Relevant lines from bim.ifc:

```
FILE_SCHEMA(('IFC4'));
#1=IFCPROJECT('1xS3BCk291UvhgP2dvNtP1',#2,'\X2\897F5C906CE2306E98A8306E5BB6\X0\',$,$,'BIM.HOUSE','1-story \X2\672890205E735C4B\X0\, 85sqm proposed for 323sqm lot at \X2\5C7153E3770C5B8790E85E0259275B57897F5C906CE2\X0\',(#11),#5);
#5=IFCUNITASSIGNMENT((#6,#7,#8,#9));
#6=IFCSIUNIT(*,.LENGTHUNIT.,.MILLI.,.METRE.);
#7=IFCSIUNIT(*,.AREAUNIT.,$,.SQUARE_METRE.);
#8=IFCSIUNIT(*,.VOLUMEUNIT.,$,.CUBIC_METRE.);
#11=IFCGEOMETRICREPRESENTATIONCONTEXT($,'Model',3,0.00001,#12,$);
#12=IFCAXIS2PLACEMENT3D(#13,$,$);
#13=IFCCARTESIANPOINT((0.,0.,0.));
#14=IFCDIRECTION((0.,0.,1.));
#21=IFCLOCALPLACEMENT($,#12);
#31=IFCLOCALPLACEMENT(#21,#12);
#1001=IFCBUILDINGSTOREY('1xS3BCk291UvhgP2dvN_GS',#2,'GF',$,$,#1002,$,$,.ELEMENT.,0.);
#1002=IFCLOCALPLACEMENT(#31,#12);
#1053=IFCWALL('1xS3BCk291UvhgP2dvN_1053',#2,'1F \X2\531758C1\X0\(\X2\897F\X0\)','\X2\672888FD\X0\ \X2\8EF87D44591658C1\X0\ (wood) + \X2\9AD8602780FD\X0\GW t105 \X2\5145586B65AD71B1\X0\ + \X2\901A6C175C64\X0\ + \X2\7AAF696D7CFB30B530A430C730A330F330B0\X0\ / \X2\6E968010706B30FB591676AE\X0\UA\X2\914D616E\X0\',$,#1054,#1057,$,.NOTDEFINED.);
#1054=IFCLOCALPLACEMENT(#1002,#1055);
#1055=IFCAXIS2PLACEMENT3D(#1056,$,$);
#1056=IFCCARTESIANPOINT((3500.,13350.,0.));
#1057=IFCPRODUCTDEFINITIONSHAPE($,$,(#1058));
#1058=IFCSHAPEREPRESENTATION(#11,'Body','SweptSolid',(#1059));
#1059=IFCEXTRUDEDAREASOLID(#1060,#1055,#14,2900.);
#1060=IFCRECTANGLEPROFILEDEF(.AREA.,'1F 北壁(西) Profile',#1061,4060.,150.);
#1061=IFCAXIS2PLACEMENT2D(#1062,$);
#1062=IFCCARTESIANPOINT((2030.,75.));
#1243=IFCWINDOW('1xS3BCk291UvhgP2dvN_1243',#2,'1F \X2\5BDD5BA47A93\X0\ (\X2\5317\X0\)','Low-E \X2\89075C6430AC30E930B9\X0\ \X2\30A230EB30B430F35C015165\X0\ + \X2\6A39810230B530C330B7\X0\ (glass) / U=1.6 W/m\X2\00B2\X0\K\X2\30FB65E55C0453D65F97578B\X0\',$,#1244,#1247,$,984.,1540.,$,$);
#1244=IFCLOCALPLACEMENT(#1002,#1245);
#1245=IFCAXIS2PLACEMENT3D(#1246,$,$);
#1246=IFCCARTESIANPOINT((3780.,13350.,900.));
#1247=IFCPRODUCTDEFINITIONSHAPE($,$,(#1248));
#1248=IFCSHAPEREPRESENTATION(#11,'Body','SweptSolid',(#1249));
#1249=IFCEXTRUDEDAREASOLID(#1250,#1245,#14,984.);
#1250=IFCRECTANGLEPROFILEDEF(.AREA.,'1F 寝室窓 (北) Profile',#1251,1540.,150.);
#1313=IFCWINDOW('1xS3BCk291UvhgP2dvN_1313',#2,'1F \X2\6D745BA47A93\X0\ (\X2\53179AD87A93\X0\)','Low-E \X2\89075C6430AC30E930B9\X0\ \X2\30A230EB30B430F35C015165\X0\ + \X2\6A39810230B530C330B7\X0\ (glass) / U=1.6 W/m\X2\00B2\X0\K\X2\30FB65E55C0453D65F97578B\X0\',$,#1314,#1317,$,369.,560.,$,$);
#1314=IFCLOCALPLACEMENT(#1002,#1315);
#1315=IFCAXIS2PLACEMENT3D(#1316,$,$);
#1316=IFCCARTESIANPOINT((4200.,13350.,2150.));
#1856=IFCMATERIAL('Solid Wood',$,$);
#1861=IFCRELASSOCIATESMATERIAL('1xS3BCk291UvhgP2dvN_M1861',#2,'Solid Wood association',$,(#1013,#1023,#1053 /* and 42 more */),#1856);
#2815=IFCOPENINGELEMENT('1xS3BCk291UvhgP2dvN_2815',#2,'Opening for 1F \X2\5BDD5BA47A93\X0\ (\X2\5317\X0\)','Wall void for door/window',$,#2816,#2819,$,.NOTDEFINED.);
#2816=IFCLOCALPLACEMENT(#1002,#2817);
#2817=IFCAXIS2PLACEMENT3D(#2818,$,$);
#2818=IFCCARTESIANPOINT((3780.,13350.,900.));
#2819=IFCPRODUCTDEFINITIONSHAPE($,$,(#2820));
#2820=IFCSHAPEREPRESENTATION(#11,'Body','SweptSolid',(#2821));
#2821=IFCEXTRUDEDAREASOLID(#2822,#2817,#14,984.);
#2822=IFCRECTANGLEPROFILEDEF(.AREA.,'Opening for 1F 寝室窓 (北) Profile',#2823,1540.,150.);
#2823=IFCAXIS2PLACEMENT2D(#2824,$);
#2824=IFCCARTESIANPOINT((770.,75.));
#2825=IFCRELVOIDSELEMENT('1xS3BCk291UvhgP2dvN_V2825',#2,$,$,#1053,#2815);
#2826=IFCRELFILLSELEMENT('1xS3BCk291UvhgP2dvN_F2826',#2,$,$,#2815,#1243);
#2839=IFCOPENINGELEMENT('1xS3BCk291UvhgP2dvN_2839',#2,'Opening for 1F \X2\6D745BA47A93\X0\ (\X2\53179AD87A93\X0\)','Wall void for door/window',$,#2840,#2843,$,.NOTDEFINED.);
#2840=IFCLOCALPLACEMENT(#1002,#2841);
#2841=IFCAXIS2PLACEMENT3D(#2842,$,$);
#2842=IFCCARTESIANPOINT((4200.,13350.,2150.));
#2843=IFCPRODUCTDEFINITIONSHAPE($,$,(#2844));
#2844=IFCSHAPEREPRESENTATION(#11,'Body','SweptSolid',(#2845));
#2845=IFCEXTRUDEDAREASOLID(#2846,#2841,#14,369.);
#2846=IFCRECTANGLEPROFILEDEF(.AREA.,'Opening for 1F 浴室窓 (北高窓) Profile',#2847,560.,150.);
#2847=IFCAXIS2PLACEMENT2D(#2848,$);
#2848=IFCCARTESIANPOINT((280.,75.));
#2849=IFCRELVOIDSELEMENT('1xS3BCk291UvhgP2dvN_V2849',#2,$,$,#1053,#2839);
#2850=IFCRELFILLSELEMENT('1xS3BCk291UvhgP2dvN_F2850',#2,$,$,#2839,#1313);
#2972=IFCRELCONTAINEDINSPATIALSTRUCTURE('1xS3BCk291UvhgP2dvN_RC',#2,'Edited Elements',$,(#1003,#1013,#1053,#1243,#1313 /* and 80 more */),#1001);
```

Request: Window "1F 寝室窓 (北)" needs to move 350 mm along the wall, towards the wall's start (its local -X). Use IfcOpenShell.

```python
import ifcopenshell
import ifcopenshell.api.geometry
import ifcopenshell.util.placement

model = ifcopenshell.open("bim.ifc")

window = model.by_guid("1xS3BCk291UvhgP2dvN_1243")
opening = window.FillsVoids[0].RelatingOpeningElement
wall = opening.VoidsElements[0].RelatingBuildingElement

wall_matrix = ifcopenshell.util.placement.get_local_placement(wall.ObjectPlacement)
shift = wall_matrix[:3, 0] * -350.0
before = ifcopenshell.util.placement.get_local_placement(window.ObjectPlacement)[:3, 3].copy()

# The window is not placed relative to its opening, so move both.
for product in (opening, window):
    matrix = ifcopenshell.util.placement.get_local_placement(product.ObjectPlacement)
    matrix[:3, 3] += shift
    ifcopenshell.api.geometry.edit_object_placement(model, product=product, matrix=matrix, is_si=False)

after = ifcopenshell.util.placement.get_local_placement(window.ObjectPlacement)[:3, 3]
print("window moved by", (after - before).round(3) + 0.0)

model.write("bim_v2.ifc")
```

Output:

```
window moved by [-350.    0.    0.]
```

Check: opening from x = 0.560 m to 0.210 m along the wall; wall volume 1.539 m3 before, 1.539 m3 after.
